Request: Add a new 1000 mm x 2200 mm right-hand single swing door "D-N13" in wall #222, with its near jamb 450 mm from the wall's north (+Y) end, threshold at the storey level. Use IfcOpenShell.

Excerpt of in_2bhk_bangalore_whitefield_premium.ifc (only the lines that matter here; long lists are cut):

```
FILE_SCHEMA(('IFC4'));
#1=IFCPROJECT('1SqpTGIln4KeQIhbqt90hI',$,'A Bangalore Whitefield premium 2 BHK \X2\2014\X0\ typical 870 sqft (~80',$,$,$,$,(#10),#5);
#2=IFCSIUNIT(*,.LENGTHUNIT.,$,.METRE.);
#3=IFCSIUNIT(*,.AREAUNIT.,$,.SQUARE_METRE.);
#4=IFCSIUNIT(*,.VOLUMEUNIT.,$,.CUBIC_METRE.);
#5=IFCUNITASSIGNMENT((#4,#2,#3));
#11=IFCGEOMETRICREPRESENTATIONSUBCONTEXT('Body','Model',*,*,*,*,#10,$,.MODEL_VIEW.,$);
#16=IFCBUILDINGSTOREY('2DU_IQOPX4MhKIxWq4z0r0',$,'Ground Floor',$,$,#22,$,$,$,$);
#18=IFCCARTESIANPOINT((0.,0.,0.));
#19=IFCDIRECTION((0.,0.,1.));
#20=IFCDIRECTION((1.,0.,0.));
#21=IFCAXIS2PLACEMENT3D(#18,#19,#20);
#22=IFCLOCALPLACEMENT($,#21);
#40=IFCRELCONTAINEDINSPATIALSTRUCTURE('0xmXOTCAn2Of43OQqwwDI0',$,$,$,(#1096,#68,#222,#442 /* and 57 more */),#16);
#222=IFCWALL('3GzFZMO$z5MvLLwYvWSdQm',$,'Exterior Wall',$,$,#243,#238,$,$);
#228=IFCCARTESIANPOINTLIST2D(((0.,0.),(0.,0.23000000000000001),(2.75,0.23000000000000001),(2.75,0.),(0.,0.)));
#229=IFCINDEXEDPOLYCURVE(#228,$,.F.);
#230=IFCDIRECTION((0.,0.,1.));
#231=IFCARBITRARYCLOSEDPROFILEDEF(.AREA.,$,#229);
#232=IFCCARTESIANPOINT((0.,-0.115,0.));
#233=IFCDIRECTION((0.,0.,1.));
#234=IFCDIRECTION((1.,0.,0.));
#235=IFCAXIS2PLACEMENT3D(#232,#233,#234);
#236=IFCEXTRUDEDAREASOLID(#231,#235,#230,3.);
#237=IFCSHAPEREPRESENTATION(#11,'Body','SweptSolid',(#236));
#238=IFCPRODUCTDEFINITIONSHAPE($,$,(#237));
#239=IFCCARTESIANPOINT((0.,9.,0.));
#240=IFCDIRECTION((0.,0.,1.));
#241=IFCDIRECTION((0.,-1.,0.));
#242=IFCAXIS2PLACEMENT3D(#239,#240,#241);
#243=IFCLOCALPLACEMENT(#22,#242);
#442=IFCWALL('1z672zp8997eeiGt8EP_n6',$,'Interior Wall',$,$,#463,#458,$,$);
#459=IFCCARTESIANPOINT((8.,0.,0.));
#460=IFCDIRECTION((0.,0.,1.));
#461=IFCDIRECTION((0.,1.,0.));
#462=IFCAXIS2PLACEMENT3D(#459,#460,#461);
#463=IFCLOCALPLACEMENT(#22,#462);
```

```python
import numpy as np
import ifcopenshell
import ifcopenshell.api.feature
import ifcopenshell.api.geometry
import ifcopenshell.api.root
import ifcopenshell.api.spatial
import ifcopenshell.geom
import ifcopenshell.util.element
import ifcopenshell.util.placement
import ifcopenshell.util.representation
import ifcopenshell.util.shape
import ifcopenshell.util.unit

model = ifcopenshell.open("in_2bhk_bangalore_whitefield_premium.ifc")
unit_scale = ifcopenshell.util.unit.calculate_unit_scale(model)
settings = ifcopenshell.geom.settings()


def volume(element):
    """Net volume in cubic metres, openings subtracted."""
    shape = ifcopenshell.geom.create_shape(settings, element)
    return ifcopenshell.util.shape.get_volume(shape.geometry)


wall = model.by_guid("3GzFZMO$z5MvLLwYvWSdQm")
storey = ifcopenshell.util.element.get_container(wall, ifc_class="IfcBuildingStorey")
context = ifcopenshell.util.representation.get_context(model, "Model", "Body", "MODEL_VIEW")
before = volume(wall)

width, height, from_end, sill = 1, 2.2, 0.45, 0.0  # metres

# The wall runs along its own X axis, and the end named is its -X end.
wall_shape = ifcopenshell.geom.create_shape(settings, wall)
x, y, z = ifcopenshell.util.shape.get_vertices(wall_shape.geometry).T
start = x.min() + from_end
face, thickness = float(y.min()), float(y.max() - y.min())
wall_matrix = ifcopenshell.util.placement.get_local_placement(wall.ObjectPlacement)
level = ifcopenshell.util.placement.get_local_placement(storey.ObjectPlacement)[2, 3]


def in_wall(x, y):
    """Placement at x, y metres in the wall's axes, at sill height."""
    matrix = wall_matrix.copy()
    matrix[:, 3] = wall_matrix @ np.array([x / unit_scale, y / unit_scale, 0.0, 1.0])
    matrix[2, 3] = level + sill / unit_scale
    return matrix


# Opening: a box that overshoots both wall faces by 50 mm.
opening = ifcopenshell.api.root.create_entity(model, ifc_class="IfcOpeningElement", predefined_type="OPENING")
box = ifcopenshell.api.geometry.add_wall_representation(
    model, context=context, length=width, height=height, thickness=thickness + 0.1
)
ifcopenshell.api.geometry.assign_representation(model, product=opening, representation=box)
ifcopenshell.api.geometry.edit_object_placement(model, product=opening, matrix=in_wall(start, face - 0.05), is_si=False)
ifcopenshell.api.feature.add_feature(model, feature=opening, element=wall)

door = ifcopenshell.api.root.create_entity(model, ifc_class="IfcDoor", name="D-N13", predefined_type="DOOR")
door.OverallWidth, door.OverallHeight = width / unit_scale, height / unit_scale
door.OperationType = "SINGLE_SWING_RIGHT"
body = ifcopenshell.api.geometry.add_door_representation(
    model,
    context=context,
    overall_width=door.OverallWidth,
    overall_height=door.OverallHeight,
    operation_type="SINGLE_SWING_RIGHT",
    lining_properties={"LiningDepth": thickness / unit_scale, "ThresholdDepth": thickness / unit_scale},
)
ifcopenshell.api.geometry.assign_representation(model, product=door, representation=body)
ifcopenshell.api.spatial.assign_container(model, products=[door], relating_structure=storey)
ifcopenshell.api.feature.add_filling(model, opening=opening, element=door)

# The lining spans the wall, so the door starts at the wall face.
ifcopenshell.api.geometry.edit_object_placement(model, product=door, matrix=in_wall(start, face), is_si=False)

after = volume(wall)

print(f"wall volume {before:.3f} -> {after:.3f} m3")

model.write("in_2bhk_bangalore_whitefield_premium-out.ifc")
```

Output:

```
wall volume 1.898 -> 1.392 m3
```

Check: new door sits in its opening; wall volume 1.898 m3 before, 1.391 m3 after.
